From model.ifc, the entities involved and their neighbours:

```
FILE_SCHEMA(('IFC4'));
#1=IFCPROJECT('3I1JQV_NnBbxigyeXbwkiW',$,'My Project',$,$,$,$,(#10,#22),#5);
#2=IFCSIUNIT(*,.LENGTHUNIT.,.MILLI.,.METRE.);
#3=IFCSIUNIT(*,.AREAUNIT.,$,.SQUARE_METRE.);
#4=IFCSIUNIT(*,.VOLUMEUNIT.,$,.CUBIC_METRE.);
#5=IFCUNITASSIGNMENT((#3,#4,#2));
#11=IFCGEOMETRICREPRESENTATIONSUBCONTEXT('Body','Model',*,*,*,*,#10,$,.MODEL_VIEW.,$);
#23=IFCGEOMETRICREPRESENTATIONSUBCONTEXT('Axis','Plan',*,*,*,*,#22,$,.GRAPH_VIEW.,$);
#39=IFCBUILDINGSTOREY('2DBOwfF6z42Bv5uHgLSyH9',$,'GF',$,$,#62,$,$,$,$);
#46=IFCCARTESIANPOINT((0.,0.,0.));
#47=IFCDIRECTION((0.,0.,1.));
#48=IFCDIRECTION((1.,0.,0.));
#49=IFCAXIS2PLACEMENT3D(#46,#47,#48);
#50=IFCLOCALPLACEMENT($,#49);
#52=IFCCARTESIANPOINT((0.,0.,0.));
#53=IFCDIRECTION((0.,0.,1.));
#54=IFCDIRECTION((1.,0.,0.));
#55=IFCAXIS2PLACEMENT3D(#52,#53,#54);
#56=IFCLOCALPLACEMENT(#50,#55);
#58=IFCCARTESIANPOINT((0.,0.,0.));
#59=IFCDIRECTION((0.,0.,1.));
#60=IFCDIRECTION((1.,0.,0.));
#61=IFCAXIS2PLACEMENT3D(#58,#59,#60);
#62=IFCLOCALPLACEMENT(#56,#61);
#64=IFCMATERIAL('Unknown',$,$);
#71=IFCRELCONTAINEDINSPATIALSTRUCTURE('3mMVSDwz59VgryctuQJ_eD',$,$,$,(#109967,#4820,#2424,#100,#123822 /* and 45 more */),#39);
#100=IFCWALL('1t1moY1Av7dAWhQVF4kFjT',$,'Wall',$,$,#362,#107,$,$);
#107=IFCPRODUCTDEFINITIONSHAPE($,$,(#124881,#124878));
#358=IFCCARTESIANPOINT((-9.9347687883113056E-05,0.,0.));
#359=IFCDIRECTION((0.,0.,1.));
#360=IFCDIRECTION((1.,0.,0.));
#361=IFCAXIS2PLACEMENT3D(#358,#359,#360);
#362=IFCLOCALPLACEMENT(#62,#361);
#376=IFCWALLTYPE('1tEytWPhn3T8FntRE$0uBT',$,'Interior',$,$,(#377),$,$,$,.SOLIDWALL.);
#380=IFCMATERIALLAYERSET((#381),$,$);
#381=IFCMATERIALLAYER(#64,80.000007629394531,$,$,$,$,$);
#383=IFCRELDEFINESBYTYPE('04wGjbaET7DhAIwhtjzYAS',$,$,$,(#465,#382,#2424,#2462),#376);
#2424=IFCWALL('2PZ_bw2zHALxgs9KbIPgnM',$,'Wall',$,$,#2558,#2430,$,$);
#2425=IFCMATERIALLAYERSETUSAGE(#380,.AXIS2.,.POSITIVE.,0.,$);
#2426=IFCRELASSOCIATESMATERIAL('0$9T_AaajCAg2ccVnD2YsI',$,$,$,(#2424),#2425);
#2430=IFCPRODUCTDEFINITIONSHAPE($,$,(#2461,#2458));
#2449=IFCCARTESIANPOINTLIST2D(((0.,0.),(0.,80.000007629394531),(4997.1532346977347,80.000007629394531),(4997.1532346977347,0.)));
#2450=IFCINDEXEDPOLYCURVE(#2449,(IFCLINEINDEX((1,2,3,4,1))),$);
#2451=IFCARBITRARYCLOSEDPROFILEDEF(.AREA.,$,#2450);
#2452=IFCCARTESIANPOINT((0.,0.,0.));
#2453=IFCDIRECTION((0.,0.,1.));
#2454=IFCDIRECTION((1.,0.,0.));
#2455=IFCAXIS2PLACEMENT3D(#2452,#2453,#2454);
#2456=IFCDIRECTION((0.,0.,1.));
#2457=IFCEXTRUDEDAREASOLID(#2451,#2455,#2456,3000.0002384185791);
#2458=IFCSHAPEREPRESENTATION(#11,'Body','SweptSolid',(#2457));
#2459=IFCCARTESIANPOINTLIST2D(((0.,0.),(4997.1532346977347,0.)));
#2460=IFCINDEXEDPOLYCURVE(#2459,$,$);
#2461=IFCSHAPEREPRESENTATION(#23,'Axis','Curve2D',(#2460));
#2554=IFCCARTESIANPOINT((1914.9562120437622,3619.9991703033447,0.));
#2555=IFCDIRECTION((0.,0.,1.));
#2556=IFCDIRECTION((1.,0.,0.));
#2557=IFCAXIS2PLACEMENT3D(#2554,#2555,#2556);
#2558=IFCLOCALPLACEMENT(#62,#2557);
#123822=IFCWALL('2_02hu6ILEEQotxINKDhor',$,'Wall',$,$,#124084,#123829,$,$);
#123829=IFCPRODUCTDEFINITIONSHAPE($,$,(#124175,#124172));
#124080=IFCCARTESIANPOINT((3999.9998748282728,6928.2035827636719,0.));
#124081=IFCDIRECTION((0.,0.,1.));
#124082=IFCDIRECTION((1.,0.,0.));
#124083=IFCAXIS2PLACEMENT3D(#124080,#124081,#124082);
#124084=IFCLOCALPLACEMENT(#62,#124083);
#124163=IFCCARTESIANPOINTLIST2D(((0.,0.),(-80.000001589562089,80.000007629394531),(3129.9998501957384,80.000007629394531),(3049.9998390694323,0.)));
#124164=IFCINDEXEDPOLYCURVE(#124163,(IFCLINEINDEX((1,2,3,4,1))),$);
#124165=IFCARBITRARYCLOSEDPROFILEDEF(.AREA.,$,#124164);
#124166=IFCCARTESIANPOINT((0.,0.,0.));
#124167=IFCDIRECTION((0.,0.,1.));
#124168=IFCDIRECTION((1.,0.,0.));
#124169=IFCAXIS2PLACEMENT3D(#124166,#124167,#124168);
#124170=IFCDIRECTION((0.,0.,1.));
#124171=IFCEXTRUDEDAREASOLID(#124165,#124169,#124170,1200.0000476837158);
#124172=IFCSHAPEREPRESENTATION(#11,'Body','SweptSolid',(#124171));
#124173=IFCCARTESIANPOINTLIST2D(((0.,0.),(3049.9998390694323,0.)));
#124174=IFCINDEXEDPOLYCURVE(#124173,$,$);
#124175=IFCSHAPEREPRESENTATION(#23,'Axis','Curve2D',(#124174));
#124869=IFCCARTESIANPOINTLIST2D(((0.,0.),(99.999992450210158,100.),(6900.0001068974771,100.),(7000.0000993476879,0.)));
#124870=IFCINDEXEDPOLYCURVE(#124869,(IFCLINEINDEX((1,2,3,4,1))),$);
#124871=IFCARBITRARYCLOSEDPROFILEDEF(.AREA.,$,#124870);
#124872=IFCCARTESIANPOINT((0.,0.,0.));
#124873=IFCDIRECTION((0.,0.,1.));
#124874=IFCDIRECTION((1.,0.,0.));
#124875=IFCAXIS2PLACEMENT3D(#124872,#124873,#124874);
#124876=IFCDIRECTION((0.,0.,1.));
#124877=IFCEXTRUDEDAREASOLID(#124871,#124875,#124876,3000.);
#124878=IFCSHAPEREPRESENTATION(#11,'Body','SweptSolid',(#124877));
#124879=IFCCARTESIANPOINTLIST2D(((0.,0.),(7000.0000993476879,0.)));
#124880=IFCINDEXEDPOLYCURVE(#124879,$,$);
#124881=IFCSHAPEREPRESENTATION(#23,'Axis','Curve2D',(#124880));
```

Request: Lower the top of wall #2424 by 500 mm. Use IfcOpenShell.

```python
import ifcopenshell
import ifcopenshell.geom
import ifcopenshell.util.representation
import ifcopenshell.util.shape

model = ifcopenshell.open("model.ifc")
settings = ifcopenshell.geom.settings()


def volume(element):
    """Net volume in cubic metres, openings subtracted."""
    shape = ifcopenshell.geom.create_shape(settings, element)
    return ifcopenshell.util.shape.get_volume(shape.geometry)


wall = model.by_guid("2PZ_bw2zHALxgs9KbIPgnM")
before = volume(wall)

body = ifcopenshell.util.representation.get_representation(wall, "Model", "Body")
solid = body.Items[0]
old_height = solid.Depth
solid.Depth -= 500.0
after = volume(wall)

print(f"height {old_height:g} -> {solid.Depth:g}, volume {before:.3f} -> {after:.3f} m3")

model.write("model_edited.ifc")
```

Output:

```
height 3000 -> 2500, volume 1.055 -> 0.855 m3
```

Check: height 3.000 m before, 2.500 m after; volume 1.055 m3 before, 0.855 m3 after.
